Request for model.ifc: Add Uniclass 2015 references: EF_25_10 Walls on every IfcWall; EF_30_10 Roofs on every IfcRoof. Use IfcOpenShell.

First a look at what the model holds.

```python
import ifcopenshell

model = ifcopenshell.open("model.ifc")
print(model.schema)
print("classifications:", [c.Name for c in model.by_type("IfcClassification")])
for ifc_class in ("IfcDoor", "IfcRoof", "IfcStair", "IfcWall", "IfcWindow"):
    print(ifc_class, len(model.by_type(ifc_class)))
```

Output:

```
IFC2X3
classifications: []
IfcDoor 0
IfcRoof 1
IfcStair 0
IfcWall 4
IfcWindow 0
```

```python
import ifcopenshell
import ifcopenshell.api.classification

model = ifcopenshell.open("model.ifc")

# IFC2X3 requires Source and Edition and has no link from the project to the system.
system = model.create_entity("IfcClassification", Source="NBS", Edition="2015", Name="Uniclass 2015")

codes = {
    "IfcWall": ("EF_25_10", "Walls"),
    "IfcRoof": ("EF_30_10", "Roofs"),
}
for ifc_class, (code, name) in codes.items():
    products = model.by_type(ifc_class)
    ifcopenshell.api.classification.add_reference(
        model, products=products, classification=system, identification=code, name=name
    )
    print(code, len(products))

model.write("model_v2.ifc")
```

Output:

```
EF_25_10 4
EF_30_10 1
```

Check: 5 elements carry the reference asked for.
